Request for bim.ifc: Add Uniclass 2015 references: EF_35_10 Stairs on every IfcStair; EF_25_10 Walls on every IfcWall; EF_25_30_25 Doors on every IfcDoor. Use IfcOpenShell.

First a look at what the model holds.

```python
import ifcopenshell

model = ifcopenshell.open("bim.ifc")
print(model.schema)
print("classifications:", [c.Name for c in model.by_type("IfcClassification")])
for ifc_class in ("IfcDoor", "IfcRoof", "IfcStair", "IfcWall", "IfcWindow"):
    print(ifc_class, len(model.by_type(ifc_class)))
```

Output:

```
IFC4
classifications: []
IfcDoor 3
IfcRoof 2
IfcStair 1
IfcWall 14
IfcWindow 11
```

```python
import ifcopenshell
import ifcopenshell.api.classification

model = ifcopenshell.open("bim.ifc")

system = ifcopenshell.api.classification.add_classification(model, classification="Uniclass 2015")

codes = {
    "IfcStair": ("EF_35_10", "Stairs"),
    "IfcWall": ("EF_25_10", "Walls"),
    "IfcDoor": ("EF_25_30_25", "Doors"),
}
for ifc_class, (code, name) in codes.items():
    products = model.by_type(ifc_class)
    ifcopenshell.api.classification.add_reference(
        model, products=products, classification=system, identification=code, name=name
    )
    print(code, len(products))

model.write("bim_edited.ifc")
```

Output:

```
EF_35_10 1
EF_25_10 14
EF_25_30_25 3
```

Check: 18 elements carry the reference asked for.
